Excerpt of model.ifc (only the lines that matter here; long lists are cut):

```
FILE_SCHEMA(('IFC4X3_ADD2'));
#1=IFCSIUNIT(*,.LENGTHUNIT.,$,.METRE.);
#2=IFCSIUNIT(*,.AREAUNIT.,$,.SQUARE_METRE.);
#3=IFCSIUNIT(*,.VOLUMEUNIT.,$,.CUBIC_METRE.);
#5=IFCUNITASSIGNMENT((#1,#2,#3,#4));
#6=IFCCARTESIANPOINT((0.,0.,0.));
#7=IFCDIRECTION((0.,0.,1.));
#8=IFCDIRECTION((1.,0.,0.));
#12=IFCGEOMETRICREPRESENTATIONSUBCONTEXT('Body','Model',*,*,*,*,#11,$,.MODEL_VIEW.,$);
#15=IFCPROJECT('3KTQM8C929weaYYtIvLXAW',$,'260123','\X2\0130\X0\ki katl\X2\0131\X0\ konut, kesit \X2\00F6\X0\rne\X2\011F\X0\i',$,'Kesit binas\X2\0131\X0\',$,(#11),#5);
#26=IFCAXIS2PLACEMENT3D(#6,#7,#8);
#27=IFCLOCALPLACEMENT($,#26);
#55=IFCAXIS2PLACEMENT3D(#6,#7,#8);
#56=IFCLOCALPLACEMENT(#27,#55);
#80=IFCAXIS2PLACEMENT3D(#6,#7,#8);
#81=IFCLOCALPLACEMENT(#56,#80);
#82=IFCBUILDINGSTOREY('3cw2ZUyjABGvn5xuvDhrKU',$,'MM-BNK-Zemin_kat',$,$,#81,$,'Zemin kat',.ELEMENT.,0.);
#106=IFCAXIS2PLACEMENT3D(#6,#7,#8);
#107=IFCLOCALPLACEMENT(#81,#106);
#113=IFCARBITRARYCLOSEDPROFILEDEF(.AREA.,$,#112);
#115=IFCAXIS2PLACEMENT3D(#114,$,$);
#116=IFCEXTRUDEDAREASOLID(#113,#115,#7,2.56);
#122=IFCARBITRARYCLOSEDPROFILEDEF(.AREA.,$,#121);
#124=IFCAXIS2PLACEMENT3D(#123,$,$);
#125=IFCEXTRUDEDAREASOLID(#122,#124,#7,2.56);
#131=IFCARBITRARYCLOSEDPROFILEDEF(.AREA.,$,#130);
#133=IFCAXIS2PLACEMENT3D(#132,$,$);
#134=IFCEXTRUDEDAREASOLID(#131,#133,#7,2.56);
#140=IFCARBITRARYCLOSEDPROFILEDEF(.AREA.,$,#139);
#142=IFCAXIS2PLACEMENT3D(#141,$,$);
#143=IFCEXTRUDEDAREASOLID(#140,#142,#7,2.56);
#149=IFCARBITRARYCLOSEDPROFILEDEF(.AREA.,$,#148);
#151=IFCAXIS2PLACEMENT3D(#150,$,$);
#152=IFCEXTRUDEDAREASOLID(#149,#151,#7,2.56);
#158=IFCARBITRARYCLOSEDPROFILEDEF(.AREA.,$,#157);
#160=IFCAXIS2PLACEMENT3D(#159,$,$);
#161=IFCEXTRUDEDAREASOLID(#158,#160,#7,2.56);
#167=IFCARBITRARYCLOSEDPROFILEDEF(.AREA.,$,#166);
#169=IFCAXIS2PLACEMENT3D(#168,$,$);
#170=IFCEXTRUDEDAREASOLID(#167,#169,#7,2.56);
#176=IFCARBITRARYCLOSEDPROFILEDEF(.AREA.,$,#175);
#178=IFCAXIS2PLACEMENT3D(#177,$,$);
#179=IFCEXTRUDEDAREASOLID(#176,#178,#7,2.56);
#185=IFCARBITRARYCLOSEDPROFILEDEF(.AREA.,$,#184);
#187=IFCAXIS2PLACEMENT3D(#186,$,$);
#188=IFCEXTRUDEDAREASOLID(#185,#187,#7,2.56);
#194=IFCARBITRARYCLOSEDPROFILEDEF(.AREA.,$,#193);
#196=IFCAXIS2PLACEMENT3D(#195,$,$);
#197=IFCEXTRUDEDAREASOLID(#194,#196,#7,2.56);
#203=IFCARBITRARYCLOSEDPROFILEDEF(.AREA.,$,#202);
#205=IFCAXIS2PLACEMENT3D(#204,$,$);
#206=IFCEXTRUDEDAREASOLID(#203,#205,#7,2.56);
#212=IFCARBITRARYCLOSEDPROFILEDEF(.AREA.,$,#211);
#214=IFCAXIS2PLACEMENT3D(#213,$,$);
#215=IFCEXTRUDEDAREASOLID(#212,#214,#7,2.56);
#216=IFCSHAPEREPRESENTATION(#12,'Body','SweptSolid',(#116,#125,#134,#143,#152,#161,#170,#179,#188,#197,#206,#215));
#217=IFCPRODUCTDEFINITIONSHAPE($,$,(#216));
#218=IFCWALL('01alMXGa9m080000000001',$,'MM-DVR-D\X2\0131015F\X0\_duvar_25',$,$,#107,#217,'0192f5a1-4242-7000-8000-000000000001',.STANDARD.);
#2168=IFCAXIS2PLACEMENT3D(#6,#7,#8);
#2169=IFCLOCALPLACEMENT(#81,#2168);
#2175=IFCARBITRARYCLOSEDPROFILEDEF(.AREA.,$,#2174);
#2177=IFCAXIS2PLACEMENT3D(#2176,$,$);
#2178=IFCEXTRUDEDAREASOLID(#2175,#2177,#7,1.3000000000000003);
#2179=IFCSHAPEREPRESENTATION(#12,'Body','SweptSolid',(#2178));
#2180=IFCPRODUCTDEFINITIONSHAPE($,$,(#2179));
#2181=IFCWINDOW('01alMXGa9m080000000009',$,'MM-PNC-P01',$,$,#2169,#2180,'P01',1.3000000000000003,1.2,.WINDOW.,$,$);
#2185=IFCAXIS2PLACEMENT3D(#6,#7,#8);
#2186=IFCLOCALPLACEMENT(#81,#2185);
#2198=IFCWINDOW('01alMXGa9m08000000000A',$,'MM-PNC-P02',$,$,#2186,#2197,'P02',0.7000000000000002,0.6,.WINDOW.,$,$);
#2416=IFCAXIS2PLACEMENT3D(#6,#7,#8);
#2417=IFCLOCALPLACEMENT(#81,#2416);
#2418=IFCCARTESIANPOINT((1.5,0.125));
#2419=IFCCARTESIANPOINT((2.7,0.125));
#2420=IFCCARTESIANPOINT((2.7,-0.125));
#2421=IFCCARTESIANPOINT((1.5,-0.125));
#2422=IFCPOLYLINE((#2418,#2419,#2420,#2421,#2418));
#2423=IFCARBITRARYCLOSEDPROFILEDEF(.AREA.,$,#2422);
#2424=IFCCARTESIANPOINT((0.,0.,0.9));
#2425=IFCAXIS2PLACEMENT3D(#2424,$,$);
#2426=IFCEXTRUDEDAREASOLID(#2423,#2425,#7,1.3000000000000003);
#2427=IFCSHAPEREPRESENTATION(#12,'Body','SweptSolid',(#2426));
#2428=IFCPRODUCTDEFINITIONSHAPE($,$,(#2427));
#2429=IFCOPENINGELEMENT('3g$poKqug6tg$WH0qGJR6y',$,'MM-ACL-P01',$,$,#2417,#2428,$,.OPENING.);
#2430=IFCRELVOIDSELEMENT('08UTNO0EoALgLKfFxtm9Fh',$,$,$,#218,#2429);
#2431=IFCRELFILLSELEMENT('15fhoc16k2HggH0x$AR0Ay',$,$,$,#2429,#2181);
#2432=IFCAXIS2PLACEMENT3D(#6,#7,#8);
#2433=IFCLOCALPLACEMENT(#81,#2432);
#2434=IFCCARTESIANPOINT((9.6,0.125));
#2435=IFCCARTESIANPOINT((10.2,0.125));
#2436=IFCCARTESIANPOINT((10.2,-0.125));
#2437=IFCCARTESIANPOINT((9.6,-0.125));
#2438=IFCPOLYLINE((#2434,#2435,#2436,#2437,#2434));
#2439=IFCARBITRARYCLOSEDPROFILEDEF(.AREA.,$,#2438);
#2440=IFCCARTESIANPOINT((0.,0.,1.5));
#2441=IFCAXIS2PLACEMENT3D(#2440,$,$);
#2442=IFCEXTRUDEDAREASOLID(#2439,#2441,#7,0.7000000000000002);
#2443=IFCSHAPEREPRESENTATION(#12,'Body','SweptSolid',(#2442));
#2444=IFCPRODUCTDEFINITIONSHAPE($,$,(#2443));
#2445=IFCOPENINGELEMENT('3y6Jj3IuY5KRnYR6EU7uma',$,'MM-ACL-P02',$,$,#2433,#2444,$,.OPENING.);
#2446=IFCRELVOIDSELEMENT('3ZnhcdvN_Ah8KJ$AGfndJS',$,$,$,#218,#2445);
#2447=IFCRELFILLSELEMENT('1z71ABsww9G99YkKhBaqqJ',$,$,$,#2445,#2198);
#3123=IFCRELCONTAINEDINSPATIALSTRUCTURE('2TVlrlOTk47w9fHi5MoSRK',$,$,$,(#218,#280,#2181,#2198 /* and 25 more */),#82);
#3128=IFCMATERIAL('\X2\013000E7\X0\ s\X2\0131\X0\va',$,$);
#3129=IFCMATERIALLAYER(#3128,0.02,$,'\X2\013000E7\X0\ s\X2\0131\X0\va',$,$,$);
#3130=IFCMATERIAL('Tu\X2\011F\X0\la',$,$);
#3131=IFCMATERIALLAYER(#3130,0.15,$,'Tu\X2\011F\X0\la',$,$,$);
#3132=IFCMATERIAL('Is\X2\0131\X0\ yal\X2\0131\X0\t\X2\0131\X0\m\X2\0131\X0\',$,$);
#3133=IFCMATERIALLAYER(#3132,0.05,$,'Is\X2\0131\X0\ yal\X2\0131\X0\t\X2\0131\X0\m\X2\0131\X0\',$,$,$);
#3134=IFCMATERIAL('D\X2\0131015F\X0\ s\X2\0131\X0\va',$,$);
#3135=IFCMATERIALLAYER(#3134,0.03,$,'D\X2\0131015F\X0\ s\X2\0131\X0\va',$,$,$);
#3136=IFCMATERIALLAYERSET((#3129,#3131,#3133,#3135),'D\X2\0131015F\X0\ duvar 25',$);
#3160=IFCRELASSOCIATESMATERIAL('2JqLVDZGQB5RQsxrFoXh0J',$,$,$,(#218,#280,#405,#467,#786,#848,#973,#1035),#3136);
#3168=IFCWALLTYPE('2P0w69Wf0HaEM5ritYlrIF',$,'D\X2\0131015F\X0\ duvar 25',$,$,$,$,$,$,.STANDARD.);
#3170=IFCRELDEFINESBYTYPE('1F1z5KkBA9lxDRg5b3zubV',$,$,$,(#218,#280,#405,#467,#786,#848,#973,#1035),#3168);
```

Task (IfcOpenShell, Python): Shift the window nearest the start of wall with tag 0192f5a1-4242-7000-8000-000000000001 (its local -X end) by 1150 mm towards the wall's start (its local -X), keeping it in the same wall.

```python
import ifcopenshell
import ifcopenshell.api.geometry
import ifcopenshell.util.placement

model = ifcopenshell.open("model.ifc")

window = model.by_id(2181)
opening = window.FillsVoids[0].RelatingOpeningElement
wall = opening.VoidsElements[0].RelatingBuildingElement

wall_matrix = ifcopenshell.util.placement.get_local_placement(wall.ObjectPlacement)
shift = wall_matrix[:3, 0] * -1.15
before = ifcopenshell.util.placement.get_local_placement(window.ObjectPlacement)[:3, 3].copy()

# The window is not placed relative to its opening, so move both.
for product in (opening, window):
    matrix = ifcopenshell.util.placement.get_local_placement(product.ObjectPlacement)
    matrix[:3, 3] += shift
    ifcopenshell.api.geometry.edit_object_placement(model, product=product, matrix=matrix, is_si=False)

after = ifcopenshell.util.placement.get_local_placement(window.ObjectPlacement)[:3, 3]
print("window moved by", (after - before).round(3) + 0.0)

model.write("model_v2.ifc")
```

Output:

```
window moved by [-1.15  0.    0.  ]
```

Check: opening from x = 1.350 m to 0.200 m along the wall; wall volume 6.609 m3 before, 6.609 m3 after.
